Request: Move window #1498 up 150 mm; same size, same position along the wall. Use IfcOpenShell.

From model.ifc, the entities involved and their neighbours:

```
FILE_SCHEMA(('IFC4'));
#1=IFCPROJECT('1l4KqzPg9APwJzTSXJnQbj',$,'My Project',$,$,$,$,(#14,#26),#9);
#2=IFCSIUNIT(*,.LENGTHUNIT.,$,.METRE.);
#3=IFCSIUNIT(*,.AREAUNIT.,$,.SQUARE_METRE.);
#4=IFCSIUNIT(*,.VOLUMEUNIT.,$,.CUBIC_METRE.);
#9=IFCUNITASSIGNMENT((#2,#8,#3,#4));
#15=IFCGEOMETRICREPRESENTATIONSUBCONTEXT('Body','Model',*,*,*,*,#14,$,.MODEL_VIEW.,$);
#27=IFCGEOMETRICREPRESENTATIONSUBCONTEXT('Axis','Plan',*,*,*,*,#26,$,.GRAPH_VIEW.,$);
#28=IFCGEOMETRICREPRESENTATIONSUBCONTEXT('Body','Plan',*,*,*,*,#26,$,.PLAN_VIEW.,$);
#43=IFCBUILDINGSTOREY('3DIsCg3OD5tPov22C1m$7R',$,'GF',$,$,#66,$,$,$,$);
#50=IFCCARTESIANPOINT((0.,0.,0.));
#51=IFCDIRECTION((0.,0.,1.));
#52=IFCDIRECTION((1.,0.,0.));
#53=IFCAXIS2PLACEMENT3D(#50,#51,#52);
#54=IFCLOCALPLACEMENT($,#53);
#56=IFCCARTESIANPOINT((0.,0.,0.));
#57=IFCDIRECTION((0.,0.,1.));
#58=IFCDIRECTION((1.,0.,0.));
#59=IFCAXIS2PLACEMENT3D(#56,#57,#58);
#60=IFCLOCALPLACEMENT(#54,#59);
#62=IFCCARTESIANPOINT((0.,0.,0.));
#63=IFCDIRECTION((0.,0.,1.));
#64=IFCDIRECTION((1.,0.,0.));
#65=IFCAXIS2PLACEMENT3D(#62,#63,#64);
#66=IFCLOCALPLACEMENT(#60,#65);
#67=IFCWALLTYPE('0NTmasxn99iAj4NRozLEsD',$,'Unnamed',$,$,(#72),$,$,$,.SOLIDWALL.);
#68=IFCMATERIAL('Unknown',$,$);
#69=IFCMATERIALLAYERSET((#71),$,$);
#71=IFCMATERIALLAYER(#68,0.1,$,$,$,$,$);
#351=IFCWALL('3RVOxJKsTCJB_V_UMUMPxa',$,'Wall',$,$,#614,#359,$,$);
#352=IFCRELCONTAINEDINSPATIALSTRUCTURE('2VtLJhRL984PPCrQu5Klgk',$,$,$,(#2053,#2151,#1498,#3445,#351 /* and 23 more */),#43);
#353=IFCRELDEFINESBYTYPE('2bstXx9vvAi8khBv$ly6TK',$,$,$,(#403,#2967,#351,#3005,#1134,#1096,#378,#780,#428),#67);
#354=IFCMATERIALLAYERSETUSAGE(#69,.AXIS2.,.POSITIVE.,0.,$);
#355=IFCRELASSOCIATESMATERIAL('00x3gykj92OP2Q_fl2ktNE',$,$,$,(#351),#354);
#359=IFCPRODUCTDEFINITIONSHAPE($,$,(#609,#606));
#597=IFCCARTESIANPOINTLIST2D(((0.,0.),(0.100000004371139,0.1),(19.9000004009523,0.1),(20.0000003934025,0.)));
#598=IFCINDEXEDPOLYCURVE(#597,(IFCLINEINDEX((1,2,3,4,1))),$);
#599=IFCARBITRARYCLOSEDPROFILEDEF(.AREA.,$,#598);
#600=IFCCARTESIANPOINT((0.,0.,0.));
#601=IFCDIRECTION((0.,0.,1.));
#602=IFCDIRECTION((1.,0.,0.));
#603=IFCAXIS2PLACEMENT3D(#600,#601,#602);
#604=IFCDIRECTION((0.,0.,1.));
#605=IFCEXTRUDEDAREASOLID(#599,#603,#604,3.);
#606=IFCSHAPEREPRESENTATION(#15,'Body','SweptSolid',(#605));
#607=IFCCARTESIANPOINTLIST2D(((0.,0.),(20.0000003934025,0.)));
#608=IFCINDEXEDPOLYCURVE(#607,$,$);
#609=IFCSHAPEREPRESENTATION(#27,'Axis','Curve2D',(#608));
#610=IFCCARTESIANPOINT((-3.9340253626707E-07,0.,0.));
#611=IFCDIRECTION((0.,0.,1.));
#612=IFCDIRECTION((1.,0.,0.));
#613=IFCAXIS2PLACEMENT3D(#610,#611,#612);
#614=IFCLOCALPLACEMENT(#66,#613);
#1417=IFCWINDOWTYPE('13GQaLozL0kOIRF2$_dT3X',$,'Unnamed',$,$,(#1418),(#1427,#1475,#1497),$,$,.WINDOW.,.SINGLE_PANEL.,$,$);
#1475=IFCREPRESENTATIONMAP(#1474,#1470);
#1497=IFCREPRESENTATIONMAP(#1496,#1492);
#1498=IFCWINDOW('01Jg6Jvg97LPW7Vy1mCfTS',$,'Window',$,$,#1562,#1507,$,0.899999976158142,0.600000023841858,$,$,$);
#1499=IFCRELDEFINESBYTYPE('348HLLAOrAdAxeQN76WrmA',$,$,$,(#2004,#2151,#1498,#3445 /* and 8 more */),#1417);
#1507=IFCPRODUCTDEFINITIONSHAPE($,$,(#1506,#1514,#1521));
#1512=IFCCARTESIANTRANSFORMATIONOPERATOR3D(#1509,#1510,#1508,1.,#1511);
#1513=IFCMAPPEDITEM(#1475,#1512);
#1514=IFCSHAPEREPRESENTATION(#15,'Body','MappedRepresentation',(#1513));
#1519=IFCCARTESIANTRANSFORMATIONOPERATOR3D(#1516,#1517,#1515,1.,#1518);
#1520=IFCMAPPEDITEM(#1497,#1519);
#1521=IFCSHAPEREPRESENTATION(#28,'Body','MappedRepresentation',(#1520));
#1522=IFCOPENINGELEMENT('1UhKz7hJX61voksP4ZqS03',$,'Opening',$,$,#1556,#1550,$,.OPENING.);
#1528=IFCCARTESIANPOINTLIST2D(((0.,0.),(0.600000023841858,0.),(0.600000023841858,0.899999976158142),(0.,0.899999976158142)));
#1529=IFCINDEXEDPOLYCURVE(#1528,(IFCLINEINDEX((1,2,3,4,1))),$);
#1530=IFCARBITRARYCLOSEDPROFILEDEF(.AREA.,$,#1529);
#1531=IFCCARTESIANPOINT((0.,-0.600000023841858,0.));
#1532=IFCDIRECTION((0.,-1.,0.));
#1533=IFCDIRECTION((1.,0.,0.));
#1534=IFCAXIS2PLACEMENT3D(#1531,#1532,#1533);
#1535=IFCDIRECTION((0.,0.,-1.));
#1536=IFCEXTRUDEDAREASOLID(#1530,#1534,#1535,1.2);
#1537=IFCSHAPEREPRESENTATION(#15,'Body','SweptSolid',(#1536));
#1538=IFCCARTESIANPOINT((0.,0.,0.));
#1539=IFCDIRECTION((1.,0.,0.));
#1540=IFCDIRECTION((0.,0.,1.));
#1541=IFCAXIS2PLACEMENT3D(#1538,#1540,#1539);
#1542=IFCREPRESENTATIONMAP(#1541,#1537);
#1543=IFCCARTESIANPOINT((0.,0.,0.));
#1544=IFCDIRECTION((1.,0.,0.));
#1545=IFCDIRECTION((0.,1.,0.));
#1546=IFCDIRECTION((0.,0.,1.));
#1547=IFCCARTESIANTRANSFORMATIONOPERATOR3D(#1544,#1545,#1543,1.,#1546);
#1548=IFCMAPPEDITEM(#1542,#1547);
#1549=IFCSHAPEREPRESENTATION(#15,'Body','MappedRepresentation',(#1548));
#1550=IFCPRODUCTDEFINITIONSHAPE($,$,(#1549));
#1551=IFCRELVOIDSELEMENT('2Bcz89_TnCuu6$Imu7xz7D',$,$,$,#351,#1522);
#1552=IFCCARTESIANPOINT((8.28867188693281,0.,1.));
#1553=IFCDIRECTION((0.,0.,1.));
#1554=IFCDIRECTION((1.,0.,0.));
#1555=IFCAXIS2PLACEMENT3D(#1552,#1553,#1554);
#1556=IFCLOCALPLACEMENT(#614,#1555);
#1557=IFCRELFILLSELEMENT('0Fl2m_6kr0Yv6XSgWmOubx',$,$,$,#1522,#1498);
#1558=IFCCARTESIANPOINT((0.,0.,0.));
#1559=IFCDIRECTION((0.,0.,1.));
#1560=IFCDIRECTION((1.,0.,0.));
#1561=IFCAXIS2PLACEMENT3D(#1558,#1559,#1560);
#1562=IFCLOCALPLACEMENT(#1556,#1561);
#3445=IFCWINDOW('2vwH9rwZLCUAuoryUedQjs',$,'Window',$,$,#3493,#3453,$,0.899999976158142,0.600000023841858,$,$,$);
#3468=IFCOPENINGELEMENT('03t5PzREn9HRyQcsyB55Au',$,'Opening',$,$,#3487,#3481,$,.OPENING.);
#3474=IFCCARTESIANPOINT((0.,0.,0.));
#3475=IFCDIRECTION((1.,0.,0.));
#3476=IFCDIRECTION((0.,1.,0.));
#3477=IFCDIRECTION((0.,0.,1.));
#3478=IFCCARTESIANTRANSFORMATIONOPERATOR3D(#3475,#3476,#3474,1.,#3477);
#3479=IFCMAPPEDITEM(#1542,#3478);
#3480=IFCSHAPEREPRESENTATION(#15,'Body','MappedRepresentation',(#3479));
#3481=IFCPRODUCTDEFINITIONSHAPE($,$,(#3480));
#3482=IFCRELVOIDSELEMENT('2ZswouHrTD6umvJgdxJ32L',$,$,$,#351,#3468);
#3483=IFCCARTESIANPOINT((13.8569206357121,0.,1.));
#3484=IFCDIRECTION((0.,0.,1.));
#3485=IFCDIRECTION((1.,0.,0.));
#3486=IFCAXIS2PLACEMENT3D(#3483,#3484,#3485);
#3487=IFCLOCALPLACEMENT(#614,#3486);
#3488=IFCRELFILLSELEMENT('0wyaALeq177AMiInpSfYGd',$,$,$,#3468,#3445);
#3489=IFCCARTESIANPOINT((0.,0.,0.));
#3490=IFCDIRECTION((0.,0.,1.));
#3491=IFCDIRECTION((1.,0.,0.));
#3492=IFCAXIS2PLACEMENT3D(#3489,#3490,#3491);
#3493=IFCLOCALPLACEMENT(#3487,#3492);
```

```python
import numpy as np
import ifcopenshell
import ifcopenshell.api.geometry
import ifcopenshell.util.placement
import ifcopenshell.util.unit

model = ifcopenshell.open("model.ifc")
unit_scale = ifcopenshell.util.unit.calculate_unit_scale(model)

window = model.by_id(1498)
opening = window.FillsVoids[0].RelatingOpeningElement
dz = 0.15 / unit_scale

shift = np.array([0.0, 0.0, dz])
# The window is placed relative to its opening, so it follows when the opening moves.
matrix = ifcopenshell.util.placement.get_local_placement(opening.ObjectPlacement)
matrix[:3, 3] += shift
ifcopenshell.api.geometry.edit_object_placement(
    model, product=opening, matrix=matrix, is_si=False, should_transform_children=True
)

print(f"moved by {dz * unit_scale:+.3f} m")

model.write("model_v2.ifc")
```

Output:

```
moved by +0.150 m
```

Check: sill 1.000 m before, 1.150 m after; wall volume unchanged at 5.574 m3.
